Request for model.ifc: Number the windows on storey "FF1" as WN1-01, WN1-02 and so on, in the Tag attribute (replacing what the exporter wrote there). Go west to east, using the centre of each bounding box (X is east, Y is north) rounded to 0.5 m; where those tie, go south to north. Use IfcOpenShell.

First a look at what the model holds.

```python
import ifcopenshell
import ifcopenshell.util.element
import ifcopenshell.util.placement

model = ifcopenshell.open("model.ifc")
print(model.schema)
storey = next(s for s in model.by_type("IfcBuildingStorey") if s.Name == "FF1")
windows = [e for e in ifcopenshell.util.element.get_decomposition(storey) if e.is_a("IfcWindow")]
for e in sorted(windows, key=lambda e: e.id()):
    origin = ifcopenshell.util.placement.get_local_placement(e.ObjectPlacement)[:3, 3]
    print(e.id(), e.Tag, e.Name, origin.round(2) + 0.0, sep=" | ")
```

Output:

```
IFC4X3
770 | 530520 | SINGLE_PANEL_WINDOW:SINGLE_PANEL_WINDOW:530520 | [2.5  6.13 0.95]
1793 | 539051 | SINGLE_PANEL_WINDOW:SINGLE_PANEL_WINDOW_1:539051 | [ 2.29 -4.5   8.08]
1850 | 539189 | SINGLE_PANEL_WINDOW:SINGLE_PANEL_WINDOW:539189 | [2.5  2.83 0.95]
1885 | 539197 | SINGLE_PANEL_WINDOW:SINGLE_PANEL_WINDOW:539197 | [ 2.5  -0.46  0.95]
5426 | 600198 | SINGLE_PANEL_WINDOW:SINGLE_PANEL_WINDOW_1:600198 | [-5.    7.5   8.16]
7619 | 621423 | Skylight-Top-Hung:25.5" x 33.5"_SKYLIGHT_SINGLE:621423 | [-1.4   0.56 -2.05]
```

```python
import ifcopenshell
import ifcopenshell.geom
import ifcopenshell.util.element
import ifcopenshell.util.shape

model = ifcopenshell.open("model.ifc")
settings = ifcopenshell.geom.settings()
settings.set("use-world-coords", True)


def centre(element):
    shape = ifcopenshell.geom.create_shape(settings, element)
    return ifcopenshell.util.shape.get_bbox_centroid(shape.geometry)


storey = next(s for s in model.by_type("IfcBuildingStorey") if s.Name == "FF1")
windows = [e for e in ifcopenshell.util.element.get_decomposition(storey) if e.is_a("IfcWindow")]

# Insertion points can sit at a corner or the storey origin, so sort by the geometry (in metres).
centres = {e: centre(e) for e in windows}
windows.sort(key=lambda e: (round(centres[e][0] / 0.5), centres[e][1]))

for i, e in enumerate(windows, start=1):
    number = f"WN1-{i:02d}"
    e.Tag = number
    print(e.id(), number)

model.write("model_rev.ifc")
```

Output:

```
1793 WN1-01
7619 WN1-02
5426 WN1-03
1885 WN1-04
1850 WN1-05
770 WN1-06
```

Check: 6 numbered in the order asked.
